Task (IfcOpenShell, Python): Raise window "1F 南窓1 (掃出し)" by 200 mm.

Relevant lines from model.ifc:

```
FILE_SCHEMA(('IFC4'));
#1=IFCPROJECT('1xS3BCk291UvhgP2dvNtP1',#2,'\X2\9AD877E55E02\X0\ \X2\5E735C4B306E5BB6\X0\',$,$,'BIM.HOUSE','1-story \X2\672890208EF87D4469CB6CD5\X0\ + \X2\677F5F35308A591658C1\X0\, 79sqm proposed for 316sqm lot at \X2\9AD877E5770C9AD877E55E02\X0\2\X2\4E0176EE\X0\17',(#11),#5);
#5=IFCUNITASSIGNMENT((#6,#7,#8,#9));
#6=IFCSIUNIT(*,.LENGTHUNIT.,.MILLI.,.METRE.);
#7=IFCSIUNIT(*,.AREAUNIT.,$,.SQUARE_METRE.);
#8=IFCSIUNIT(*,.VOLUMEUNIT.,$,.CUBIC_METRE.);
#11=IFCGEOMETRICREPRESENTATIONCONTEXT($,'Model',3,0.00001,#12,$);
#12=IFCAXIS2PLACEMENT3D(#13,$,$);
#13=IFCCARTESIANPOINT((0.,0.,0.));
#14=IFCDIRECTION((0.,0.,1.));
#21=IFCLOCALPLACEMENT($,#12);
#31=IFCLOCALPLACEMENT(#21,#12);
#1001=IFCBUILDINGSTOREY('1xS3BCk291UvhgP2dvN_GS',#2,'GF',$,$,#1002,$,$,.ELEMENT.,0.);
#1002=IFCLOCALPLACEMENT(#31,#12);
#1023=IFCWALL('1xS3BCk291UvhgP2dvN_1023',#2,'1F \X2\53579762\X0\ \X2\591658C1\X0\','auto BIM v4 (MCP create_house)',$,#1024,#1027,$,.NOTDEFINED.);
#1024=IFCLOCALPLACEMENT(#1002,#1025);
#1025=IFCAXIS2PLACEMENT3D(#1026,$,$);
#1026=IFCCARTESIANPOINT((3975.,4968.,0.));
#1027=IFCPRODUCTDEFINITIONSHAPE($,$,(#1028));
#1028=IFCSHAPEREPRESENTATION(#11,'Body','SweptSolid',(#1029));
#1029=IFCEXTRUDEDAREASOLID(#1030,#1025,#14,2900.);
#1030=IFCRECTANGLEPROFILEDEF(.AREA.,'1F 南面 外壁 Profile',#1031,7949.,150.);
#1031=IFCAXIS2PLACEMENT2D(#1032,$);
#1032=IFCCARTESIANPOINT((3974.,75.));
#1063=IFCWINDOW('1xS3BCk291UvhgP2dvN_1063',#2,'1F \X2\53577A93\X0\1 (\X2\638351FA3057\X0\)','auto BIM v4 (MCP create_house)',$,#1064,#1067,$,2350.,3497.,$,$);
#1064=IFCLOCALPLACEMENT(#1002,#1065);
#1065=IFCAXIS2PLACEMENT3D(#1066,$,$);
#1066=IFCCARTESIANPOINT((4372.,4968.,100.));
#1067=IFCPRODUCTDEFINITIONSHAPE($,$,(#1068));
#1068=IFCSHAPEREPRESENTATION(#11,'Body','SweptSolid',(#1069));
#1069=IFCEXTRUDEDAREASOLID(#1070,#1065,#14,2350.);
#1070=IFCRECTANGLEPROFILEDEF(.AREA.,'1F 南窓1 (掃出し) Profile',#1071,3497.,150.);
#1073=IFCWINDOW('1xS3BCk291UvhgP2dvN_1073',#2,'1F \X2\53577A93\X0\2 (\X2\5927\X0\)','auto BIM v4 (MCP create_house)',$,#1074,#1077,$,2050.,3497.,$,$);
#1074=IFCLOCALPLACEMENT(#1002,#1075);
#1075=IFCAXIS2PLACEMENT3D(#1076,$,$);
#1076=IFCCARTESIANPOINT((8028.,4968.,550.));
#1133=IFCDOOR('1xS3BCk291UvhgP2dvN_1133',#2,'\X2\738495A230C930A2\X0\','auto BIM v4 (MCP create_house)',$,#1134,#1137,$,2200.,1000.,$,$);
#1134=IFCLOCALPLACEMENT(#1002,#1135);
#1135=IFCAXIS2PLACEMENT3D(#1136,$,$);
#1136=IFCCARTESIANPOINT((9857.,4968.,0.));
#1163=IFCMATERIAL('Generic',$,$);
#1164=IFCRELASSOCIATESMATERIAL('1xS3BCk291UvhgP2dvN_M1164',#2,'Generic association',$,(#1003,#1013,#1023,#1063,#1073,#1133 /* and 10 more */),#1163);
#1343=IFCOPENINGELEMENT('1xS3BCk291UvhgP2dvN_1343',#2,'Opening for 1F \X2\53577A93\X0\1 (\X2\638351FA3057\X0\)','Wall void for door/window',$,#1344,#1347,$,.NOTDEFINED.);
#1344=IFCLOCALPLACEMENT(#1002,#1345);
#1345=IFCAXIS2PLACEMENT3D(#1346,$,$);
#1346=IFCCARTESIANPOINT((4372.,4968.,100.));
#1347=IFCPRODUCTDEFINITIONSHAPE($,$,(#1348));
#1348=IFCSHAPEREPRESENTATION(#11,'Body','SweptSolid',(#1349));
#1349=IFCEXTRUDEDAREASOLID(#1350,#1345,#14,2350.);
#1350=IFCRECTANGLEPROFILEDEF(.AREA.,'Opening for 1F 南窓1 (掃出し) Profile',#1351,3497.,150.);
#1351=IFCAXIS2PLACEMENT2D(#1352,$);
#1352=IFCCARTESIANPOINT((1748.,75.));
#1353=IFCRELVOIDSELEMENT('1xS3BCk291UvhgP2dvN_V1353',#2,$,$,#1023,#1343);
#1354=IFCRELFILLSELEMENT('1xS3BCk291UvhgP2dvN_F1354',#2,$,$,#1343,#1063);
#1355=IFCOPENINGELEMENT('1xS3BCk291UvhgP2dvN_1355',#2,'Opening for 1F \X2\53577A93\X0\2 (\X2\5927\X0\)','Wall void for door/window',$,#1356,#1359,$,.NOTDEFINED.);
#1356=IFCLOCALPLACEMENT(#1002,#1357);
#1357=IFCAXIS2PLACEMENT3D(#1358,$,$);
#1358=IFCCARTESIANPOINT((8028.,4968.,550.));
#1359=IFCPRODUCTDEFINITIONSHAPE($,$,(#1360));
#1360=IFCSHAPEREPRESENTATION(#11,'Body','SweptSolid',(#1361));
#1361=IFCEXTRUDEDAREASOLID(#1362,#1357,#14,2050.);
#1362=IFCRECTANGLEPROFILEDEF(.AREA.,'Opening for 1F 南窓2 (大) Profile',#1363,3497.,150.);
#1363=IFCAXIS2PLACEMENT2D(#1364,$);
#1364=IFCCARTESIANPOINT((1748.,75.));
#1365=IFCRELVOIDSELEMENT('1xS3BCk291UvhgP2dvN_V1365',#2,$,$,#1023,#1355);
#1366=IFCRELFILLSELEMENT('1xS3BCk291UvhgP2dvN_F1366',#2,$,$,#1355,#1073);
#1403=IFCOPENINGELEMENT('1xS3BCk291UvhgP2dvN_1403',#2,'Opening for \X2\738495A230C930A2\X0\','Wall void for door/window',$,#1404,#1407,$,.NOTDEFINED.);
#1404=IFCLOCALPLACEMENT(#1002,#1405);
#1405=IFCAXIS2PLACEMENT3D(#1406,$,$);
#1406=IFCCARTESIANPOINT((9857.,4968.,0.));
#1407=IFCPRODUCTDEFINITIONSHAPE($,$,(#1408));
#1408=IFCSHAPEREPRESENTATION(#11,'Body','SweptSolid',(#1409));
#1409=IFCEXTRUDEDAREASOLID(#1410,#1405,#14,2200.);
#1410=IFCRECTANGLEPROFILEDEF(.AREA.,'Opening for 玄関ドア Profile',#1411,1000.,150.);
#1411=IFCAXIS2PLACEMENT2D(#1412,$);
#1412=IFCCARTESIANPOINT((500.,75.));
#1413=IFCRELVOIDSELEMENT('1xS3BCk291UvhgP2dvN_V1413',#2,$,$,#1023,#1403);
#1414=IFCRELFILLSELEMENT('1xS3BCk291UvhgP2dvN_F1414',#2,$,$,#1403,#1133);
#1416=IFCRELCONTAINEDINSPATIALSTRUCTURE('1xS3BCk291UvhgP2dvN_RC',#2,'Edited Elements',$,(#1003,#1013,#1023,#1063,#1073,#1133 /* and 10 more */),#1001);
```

```python
import numpy as np
import ifcopenshell
import ifcopenshell.api.geometry
import ifcopenshell.util.placement
import ifcopenshell.util.unit

model = ifcopenshell.open("model.ifc")
unit_scale = ifcopenshell.util.unit.calculate_unit_scale(model)

window = model.by_guid("1xS3BCk291UvhgP2dvN_1063")
opening = window.FillsVoids[0].RelatingOpeningElement
dz = 200.0

shift = np.array([0.0, 0.0, dz])
# The window is not placed relative to its opening, so move both.
for product in (opening, window):
    matrix = ifcopenshell.util.placement.get_local_placement(product.ObjectPlacement)
    matrix[:3, 3] += shift
    ifcopenshell.api.geometry.edit_object_placement(model, product=product, matrix=matrix, is_si=False)

print(f"moved by {dz * unit_scale:+.3f} m")

model.write("model_rev.ifc")
```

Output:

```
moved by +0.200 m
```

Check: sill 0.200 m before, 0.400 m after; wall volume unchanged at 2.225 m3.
